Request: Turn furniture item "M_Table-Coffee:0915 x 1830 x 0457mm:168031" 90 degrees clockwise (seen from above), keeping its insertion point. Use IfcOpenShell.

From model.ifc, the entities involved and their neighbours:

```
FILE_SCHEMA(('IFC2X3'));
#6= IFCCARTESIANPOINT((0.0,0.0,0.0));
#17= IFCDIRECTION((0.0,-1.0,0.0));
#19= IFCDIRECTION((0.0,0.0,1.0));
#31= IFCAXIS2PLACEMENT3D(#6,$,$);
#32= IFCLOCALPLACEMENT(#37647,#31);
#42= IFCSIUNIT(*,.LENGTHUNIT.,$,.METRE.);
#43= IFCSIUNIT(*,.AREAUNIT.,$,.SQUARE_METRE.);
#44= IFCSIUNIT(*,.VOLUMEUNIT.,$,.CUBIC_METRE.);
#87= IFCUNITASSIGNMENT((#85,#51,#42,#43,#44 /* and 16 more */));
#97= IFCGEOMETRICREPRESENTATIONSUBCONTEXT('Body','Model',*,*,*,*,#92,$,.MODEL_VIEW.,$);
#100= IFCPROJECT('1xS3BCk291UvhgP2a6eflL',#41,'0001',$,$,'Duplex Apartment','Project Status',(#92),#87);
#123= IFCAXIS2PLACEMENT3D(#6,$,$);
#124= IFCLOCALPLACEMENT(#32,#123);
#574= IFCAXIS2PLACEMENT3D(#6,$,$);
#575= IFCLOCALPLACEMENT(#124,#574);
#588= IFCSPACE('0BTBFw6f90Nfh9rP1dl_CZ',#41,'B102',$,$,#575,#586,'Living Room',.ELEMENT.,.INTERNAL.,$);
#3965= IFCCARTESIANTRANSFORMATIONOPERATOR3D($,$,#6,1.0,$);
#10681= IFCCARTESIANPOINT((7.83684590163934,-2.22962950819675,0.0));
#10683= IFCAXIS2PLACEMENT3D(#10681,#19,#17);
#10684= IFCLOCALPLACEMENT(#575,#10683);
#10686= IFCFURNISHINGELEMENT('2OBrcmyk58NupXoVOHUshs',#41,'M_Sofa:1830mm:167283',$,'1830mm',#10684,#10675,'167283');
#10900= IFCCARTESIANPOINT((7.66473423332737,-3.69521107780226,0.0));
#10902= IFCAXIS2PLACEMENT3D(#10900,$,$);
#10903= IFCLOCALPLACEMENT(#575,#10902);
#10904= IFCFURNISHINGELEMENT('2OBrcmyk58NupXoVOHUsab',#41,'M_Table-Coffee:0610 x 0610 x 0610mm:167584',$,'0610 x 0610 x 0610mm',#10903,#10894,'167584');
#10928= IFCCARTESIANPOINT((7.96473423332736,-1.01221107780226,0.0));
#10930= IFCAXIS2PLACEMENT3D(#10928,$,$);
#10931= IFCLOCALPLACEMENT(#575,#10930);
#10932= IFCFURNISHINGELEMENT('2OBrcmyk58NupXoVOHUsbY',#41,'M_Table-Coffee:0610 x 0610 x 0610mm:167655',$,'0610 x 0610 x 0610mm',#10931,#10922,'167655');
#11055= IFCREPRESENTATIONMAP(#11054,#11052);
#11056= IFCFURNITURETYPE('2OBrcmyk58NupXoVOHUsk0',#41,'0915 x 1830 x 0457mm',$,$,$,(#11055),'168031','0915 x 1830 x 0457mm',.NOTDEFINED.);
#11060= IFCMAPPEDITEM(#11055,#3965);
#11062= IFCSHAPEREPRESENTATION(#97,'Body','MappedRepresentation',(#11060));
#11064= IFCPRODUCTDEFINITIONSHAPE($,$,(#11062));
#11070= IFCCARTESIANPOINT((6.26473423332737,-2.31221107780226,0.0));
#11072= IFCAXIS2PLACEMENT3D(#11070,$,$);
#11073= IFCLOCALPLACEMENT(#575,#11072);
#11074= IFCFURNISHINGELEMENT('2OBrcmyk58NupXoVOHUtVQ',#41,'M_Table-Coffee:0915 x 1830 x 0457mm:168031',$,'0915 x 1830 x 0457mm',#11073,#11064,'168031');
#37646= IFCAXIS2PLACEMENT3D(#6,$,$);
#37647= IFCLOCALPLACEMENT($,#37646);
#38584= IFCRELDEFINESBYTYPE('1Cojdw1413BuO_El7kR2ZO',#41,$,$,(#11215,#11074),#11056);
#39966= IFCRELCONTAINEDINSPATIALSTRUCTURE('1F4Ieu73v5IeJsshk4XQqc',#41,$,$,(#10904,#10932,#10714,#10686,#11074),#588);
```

```python
import ifcopenshell
import ifcopenshell.api.geometry
import ifcopenshell.util.placement

model = ifcopenshell.open("model.ifc")

item = model.by_id(11074)
matrix = ifcopenshell.util.placement.get_local_placement(item.ObjectPlacement)
matrix = matrix @ ifcopenshell.util.placement.rotation(-90, "Z")
ifcopenshell.api.geometry.edit_object_placement(model, product=item, matrix=matrix, is_si=False)

print(ifcopenshell.util.placement.get_local_placement(item.ObjectPlacement).round(3) + 0.0)

model.write("model_updated.ifc")
```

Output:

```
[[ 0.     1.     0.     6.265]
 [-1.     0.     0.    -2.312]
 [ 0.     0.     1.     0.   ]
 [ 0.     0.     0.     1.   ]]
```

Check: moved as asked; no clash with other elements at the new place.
